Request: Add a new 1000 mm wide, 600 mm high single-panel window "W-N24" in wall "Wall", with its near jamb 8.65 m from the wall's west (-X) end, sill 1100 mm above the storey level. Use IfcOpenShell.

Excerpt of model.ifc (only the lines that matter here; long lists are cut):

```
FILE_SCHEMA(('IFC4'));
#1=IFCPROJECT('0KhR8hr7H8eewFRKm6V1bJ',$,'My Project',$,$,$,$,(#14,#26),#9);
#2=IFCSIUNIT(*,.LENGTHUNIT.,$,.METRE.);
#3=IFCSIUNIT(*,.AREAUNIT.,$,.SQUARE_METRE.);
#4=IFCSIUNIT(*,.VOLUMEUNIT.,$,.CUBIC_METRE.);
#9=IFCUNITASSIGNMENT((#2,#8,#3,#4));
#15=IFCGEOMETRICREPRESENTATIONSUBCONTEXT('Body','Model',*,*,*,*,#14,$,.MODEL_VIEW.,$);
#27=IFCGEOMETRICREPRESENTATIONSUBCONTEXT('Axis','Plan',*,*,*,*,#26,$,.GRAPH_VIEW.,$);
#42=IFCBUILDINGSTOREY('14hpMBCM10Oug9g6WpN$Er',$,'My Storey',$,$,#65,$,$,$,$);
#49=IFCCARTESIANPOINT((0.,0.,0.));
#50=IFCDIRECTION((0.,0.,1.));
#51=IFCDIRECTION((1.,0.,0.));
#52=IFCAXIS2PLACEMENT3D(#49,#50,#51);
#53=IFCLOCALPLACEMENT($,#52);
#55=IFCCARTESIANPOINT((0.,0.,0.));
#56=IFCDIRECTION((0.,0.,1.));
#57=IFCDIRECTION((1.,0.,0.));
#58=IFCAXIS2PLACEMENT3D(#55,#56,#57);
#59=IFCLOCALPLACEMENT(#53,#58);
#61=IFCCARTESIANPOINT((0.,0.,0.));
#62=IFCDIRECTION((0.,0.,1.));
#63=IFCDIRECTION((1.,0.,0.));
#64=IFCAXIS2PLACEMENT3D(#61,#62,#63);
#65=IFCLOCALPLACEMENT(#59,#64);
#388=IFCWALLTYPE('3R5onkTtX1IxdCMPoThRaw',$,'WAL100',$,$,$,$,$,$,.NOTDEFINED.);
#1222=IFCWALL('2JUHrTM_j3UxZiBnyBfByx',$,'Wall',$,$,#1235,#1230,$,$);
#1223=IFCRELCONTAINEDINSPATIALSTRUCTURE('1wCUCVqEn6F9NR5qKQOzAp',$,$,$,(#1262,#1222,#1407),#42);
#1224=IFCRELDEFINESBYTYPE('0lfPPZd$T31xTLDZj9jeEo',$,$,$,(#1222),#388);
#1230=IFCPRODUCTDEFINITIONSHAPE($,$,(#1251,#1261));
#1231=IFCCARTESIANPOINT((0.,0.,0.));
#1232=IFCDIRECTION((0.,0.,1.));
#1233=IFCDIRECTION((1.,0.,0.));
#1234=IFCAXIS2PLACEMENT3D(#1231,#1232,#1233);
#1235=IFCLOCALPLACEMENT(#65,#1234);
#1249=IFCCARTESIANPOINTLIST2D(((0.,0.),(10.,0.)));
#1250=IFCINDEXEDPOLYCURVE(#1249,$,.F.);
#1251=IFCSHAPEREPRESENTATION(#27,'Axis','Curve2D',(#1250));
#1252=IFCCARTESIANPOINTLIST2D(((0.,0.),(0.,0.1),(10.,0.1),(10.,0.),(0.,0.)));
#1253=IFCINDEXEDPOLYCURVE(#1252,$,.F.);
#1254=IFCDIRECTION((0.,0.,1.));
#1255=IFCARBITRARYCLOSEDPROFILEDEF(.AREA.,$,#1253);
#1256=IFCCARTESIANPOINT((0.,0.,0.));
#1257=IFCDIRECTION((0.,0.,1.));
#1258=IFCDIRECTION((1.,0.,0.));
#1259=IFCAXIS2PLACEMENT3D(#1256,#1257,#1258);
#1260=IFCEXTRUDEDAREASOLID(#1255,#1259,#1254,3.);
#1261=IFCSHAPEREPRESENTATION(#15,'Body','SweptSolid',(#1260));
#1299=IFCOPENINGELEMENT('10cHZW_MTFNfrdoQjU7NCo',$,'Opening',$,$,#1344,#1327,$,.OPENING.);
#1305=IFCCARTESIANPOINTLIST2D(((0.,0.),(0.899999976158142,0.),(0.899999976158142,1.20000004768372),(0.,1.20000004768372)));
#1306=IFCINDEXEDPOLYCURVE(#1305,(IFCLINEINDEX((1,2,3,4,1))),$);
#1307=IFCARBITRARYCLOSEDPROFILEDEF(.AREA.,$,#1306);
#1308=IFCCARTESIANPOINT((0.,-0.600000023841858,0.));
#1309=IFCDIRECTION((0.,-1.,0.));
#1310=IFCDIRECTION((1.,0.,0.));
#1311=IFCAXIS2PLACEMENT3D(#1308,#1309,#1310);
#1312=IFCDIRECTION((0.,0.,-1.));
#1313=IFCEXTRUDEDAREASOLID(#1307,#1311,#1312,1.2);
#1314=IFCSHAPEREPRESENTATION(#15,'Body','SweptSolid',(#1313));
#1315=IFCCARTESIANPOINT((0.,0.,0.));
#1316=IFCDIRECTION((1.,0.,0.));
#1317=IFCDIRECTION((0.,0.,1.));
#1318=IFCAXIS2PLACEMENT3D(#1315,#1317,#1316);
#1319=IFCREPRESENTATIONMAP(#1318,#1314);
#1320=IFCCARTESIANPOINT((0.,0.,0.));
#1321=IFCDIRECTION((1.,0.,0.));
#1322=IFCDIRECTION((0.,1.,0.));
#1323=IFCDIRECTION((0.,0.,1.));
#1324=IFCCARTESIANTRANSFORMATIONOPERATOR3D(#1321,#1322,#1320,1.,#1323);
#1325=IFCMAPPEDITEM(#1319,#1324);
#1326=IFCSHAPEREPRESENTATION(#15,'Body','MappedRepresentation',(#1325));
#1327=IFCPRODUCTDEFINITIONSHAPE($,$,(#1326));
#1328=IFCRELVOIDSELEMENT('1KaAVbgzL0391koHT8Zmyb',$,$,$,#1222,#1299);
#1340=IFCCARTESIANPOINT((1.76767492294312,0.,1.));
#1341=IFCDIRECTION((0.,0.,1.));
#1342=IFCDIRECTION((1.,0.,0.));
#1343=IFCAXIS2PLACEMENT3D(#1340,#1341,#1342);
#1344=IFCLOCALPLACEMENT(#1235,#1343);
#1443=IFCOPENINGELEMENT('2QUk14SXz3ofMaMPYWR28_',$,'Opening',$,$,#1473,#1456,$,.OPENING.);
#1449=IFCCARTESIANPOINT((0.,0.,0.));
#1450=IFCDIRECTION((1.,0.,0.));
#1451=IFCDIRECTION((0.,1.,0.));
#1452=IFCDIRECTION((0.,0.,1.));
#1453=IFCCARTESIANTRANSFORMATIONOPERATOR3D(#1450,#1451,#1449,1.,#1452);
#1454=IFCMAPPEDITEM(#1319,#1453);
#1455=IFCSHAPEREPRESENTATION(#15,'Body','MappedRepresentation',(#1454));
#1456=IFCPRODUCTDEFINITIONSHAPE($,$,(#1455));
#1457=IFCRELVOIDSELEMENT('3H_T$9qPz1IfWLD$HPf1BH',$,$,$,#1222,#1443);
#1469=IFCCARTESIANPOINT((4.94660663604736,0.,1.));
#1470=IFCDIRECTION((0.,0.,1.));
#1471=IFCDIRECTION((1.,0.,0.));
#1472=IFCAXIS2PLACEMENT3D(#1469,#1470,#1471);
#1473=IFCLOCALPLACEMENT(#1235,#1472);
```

```python
import numpy as np
import ifcopenshell
import ifcopenshell.api.feature
import ifcopenshell.api.geometry
import ifcopenshell.api.root
import ifcopenshell.api.spatial
import ifcopenshell.geom
import ifcopenshell.util.element
import ifcopenshell.util.placement
import ifcopenshell.util.representation
import ifcopenshell.util.shape
import ifcopenshell.util.unit

model = ifcopenshell.open("model.ifc")
unit_scale = ifcopenshell.util.unit.calculate_unit_scale(model)
settings = ifcopenshell.geom.settings()


def volume(element):
    """Net volume in cubic metres, openings subtracted."""
    shape = ifcopenshell.geom.create_shape(settings, element)
    return ifcopenshell.util.shape.get_volume(shape.geometry)


wall = model.by_guid("2JUHrTM_j3UxZiBnyBfByx")
storey = ifcopenshell.util.element.get_container(wall, ifc_class="IfcBuildingStorey")
context = ifcopenshell.util.representation.get_context(model, "Model", "Body", "MODEL_VIEW")
before = volume(wall)

width, height, from_end, sill = 1, 0.6, 8.65, 1.1  # metres

# The wall runs along its own X axis, and the end named is its -X end.
wall_shape = ifcopenshell.geom.create_shape(settings, wall)
x, y, z = ifcopenshell.util.shape.get_vertices(wall_shape.geometry).T
start = x.min() + from_end
face, thickness = float(y.min()), float(y.max() - y.min())
wall_matrix = ifcopenshell.util.placement.get_local_placement(wall.ObjectPlacement)
level = ifcopenshell.util.placement.get_local_placement(storey.ObjectPlacement)[2, 3]


def in_wall(x, y):
    """Placement at x, y metres in the wall's axes, at sill height."""
    matrix = wall_matrix.copy()
    matrix[:, 3] = wall_matrix @ np.array([x / unit_scale, y / unit_scale, 0.0, 1.0])
    matrix[2, 3] = level + sill / unit_scale
    return matrix


# Opening: a box that overshoots both wall faces by 50 mm.
opening = ifcopenshell.api.root.create_entity(model, ifc_class="IfcOpeningElement", predefined_type="OPENING")
box = ifcopenshell.api.geometry.add_wall_representation(
    model, context=context, length=width, height=height, thickness=thickness + 0.1
)
ifcopenshell.api.geometry.assign_representation(model, product=opening, representation=box)
ifcopenshell.api.geometry.edit_object_placement(model, product=opening, matrix=in_wall(start, face - 0.05), is_si=False)
ifcopenshell.api.feature.add_feature(model, feature=opening, element=wall)

window = ifcopenshell.api.root.create_entity(model, ifc_class="IfcWindow", name="W-N24", predefined_type="WINDOW")
window.OverallWidth, window.OverallHeight = width / unit_scale, height / unit_scale
window.PartitioningType = "SINGLE_PANEL"
body = ifcopenshell.api.geometry.add_window_representation(
    model,
    context=context,
    overall_width=window.OverallWidth,
    overall_height=window.OverallHeight,
    partition_type="SINGLE_PANEL",
)
ifcopenshell.api.geometry.assign_representation(model, product=window, representation=body)
ifcopenshell.api.spatial.assign_container(model, products=[window], relating_structure=storey)
ifcopenshell.api.feature.add_filling(model, opening=opening, element=window)

# Centre the window in the wall's thickness.
ifcopenshell.api.geometry.edit_object_placement(model, product=window, matrix=in_wall(start, face), is_si=False)
window_shape = ifcopenshell.geom.create_shape(settings, window)
depth = ifcopenshell.util.shape.get_vertices(window_shape.geometry)[:, 1]
offset = face + thickness / 2 - (depth.min() + depth.max()) / 2
ifcopenshell.api.geometry.edit_object_placement(model, product=window, matrix=in_wall(start, offset), is_si=False)

after = volume(wall)

print(f"wall volume {before:.3f} -> {after:.3f} m3")

model.write("model_updated.ifc")
```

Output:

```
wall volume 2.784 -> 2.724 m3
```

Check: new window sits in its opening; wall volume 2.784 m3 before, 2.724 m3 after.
